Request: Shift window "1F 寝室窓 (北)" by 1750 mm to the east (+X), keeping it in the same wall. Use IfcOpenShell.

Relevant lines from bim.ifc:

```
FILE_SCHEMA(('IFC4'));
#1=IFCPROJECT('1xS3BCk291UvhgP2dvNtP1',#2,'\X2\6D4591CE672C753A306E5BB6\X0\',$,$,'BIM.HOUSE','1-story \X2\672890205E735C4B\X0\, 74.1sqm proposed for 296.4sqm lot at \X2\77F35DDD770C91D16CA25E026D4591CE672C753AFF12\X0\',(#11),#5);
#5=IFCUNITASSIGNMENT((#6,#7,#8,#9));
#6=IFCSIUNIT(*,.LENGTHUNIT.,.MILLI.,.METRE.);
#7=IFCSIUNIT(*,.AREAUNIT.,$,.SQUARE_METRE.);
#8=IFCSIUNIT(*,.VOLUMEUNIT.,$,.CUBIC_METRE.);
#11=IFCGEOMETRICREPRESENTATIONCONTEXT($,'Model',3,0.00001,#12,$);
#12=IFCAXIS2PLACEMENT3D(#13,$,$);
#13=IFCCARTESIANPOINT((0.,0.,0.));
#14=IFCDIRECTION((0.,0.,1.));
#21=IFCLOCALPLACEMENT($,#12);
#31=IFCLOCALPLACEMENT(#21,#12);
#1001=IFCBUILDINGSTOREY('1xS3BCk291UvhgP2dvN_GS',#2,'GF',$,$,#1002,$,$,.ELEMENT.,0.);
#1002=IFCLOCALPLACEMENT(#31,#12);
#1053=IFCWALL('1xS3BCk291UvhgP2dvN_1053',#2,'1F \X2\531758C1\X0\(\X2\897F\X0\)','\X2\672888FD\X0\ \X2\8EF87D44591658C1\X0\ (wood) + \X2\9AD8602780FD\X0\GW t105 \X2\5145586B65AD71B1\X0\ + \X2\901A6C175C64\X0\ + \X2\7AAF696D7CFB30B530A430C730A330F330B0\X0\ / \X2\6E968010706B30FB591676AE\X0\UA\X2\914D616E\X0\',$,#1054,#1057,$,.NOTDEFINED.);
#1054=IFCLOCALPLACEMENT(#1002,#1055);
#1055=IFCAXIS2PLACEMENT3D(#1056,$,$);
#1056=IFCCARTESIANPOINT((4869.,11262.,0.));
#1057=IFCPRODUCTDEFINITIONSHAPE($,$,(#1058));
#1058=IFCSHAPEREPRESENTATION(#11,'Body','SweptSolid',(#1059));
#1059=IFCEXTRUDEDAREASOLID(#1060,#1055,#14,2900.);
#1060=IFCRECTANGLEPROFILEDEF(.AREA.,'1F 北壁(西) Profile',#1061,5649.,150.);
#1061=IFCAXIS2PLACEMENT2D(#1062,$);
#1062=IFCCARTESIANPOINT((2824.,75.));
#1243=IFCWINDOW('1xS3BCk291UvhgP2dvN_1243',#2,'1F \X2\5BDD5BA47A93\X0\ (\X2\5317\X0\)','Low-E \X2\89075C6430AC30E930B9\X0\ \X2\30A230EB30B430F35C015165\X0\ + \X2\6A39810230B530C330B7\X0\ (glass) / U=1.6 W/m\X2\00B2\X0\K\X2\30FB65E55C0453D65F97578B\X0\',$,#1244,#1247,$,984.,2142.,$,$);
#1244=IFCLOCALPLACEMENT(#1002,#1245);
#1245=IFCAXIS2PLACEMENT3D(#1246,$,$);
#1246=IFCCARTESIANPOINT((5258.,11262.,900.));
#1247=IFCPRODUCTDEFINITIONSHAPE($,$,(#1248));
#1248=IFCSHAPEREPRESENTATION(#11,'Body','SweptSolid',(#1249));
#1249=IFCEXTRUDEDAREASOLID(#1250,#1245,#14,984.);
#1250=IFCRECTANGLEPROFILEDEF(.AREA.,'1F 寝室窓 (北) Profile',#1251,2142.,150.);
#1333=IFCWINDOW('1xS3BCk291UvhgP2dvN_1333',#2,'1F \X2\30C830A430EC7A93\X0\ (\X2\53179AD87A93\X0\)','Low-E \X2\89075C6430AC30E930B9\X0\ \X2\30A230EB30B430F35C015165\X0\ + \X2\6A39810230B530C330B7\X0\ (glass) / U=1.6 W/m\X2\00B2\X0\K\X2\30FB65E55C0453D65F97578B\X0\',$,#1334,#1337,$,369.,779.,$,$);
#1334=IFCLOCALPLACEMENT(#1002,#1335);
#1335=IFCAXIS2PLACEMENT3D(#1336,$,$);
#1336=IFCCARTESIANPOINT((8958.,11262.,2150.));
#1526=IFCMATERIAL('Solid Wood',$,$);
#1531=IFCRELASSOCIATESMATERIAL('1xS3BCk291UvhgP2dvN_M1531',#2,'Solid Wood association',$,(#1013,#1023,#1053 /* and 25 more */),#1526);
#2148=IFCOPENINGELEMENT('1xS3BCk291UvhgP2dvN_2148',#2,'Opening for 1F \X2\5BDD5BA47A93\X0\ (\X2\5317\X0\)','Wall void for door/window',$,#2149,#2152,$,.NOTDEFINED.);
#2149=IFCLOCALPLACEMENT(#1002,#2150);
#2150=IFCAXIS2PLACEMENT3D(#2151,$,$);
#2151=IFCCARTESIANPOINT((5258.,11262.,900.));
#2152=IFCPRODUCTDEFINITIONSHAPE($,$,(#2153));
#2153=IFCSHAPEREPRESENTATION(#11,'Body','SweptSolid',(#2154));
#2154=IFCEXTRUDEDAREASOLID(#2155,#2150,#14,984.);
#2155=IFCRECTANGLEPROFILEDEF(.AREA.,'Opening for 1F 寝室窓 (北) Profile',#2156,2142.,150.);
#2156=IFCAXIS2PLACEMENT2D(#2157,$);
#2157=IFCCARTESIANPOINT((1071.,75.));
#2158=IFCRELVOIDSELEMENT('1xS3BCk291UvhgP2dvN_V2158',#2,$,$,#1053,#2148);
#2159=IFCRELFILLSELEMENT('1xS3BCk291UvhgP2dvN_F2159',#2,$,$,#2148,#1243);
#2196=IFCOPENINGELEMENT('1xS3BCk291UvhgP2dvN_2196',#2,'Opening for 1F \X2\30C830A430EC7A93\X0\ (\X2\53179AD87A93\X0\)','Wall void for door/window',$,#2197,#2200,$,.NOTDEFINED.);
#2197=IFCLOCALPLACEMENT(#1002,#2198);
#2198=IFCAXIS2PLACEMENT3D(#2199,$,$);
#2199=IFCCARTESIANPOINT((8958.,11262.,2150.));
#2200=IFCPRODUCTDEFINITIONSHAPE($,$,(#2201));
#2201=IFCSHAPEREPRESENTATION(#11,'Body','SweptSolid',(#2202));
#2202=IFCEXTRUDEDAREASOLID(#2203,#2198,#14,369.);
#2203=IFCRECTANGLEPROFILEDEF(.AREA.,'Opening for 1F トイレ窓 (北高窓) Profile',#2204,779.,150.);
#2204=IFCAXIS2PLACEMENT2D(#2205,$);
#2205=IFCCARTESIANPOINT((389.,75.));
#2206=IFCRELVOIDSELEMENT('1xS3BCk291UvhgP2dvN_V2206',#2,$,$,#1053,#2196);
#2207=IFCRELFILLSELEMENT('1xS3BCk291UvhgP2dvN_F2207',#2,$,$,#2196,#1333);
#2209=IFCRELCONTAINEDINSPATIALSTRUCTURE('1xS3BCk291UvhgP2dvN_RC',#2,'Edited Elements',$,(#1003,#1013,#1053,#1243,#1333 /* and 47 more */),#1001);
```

```python
import ifcopenshell
import ifcopenshell.api.geometry
import ifcopenshell.util.placement
import ifcopenshell.util.unit

model = ifcopenshell.open("bim.ifc")
unit_scale = ifcopenshell.util.unit.calculate_unit_scale(model)

window = model.by_guid("1xS3BCk291UvhgP2dvN_1243")
opening = window.FillsVoids[0].RelatingOpeningElement
wall = opening.VoidsElements[0].RelatingBuildingElement

wall_matrix = ifcopenshell.util.placement.get_local_placement(wall.ObjectPlacement)
shift = wall_matrix[:3, 0] * 1.75 / unit_scale
before = ifcopenshell.util.placement.get_local_placement(window.ObjectPlacement)[:3, 3].copy()

# The window is not placed relative to its opening, so move both.
for product in (opening, window):
    matrix = ifcopenshell.util.placement.get_local_placement(product.ObjectPlacement)
    matrix[:3, 3] += shift
    ifcopenshell.api.geometry.edit_object_placement(model, product=product, matrix=matrix, is_si=False)

after = ifcopenshell.util.placement.get_local_placement(window.ObjectPlacement)[:3, 3]
print("window moved by", (after - before).round(3) + 0.0)

model.write("bim_v2.ifc")
```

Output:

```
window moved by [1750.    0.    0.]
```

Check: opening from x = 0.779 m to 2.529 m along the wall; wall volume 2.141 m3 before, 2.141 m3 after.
